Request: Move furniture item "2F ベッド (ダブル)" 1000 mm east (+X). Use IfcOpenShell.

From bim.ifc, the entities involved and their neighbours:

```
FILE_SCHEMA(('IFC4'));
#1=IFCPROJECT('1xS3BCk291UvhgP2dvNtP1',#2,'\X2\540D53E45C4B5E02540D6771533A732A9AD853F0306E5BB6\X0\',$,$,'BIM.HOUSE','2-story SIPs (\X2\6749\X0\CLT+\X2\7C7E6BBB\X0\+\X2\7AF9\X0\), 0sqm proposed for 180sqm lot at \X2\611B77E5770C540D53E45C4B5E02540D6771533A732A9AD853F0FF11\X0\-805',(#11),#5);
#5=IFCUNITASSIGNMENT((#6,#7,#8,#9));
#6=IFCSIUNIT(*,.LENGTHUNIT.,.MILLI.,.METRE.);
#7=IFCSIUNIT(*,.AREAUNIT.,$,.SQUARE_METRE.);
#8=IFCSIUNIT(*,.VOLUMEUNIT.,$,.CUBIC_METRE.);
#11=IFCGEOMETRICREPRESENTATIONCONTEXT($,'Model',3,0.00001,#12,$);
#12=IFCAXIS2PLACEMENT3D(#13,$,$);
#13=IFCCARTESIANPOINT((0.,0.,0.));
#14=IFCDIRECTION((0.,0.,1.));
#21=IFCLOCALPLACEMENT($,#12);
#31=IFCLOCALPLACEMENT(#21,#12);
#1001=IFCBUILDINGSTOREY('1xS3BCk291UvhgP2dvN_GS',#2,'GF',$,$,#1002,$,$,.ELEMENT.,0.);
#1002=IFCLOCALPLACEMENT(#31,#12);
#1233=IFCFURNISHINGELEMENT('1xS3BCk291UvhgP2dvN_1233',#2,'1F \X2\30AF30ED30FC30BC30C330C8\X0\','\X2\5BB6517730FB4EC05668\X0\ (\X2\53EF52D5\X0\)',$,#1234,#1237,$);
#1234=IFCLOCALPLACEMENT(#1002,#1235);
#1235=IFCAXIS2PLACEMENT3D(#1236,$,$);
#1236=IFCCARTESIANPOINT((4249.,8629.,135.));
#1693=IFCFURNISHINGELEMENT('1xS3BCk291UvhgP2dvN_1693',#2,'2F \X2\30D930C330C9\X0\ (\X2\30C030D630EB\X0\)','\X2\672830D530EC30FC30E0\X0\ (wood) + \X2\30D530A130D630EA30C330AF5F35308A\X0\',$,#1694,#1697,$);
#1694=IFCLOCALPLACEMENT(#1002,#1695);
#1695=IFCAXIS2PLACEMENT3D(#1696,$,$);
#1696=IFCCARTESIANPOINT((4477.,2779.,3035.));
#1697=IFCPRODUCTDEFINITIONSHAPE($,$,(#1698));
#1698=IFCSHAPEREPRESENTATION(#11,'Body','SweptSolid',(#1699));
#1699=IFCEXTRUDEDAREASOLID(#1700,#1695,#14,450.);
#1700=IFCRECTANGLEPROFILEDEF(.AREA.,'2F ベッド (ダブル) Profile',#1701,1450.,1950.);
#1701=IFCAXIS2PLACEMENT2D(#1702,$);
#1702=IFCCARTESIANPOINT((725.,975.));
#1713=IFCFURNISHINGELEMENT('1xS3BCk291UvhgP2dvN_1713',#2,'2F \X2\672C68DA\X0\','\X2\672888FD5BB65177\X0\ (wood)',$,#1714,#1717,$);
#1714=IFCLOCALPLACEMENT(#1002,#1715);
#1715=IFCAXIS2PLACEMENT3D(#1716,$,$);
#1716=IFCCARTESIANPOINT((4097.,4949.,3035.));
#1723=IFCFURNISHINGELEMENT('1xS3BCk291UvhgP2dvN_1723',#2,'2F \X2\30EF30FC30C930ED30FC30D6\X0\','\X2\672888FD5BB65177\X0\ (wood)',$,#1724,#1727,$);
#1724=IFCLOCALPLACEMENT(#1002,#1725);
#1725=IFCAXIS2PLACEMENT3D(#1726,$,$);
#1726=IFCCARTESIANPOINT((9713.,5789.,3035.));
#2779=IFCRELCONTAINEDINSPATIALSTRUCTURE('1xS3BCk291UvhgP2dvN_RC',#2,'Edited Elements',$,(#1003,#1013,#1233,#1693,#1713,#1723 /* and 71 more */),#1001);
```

```python
import ifcopenshell
import ifcopenshell.api.geometry
import ifcopenshell.util.placement

model = ifcopenshell.open("bim.ifc")

item = model.by_guid("1xS3BCk291UvhgP2dvN_1693")
matrix = ifcopenshell.util.placement.get_local_placement(item.ObjectPlacement)
matrix[0, 3] += 1000.0
ifcopenshell.api.geometry.edit_object_placement(model, product=item, matrix=matrix, is_si=False)

print(ifcopenshell.util.placement.get_local_placement(item.ObjectPlacement).round(3) + 0.0)

model.write("bim_updated.ifc")
```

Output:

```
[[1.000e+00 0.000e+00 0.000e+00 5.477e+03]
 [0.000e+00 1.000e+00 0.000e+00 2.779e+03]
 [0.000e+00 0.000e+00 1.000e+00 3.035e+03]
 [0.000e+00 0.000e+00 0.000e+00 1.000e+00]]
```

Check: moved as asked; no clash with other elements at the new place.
